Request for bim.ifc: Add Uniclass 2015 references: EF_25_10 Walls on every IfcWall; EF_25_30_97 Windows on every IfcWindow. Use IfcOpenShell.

First a look at what the model holds.

```python
import ifcopenshell

model = ifcopenshell.open("bim.ifc")
print(model.schema)
print("classifications:", [c.Name for c in model.by_type("IfcClassification")])
for ifc_class in ("IfcDoor", "IfcRoof", "IfcStair", "IfcWall", "IfcWindow"):
    print(ifc_class, len(model.by_type(ifc_class)))
```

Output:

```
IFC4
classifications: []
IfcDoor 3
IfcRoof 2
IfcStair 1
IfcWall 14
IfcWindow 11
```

```python
import ifcopenshell
import ifcopenshell.api.classification

model = ifcopenshell.open("bim.ifc")

system = ifcopenshell.api.classification.add_classification(model, classification="Uniclass 2015")

codes = {
    "IfcWall": ("EF_25_10", "Walls"),
    "IfcWindow": ("EF_25_30_97", "Windows"),
}
for ifc_class, (code, name) in codes.items():
    products = model.by_type(ifc_class)
    ifcopenshell.api.classification.add_reference(
        model, products=products, classification=system, identification=code, name=name
    )
    print(code, len(products))

model.write("bim_updated.ifc")
```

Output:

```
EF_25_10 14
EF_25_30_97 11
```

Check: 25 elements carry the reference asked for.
